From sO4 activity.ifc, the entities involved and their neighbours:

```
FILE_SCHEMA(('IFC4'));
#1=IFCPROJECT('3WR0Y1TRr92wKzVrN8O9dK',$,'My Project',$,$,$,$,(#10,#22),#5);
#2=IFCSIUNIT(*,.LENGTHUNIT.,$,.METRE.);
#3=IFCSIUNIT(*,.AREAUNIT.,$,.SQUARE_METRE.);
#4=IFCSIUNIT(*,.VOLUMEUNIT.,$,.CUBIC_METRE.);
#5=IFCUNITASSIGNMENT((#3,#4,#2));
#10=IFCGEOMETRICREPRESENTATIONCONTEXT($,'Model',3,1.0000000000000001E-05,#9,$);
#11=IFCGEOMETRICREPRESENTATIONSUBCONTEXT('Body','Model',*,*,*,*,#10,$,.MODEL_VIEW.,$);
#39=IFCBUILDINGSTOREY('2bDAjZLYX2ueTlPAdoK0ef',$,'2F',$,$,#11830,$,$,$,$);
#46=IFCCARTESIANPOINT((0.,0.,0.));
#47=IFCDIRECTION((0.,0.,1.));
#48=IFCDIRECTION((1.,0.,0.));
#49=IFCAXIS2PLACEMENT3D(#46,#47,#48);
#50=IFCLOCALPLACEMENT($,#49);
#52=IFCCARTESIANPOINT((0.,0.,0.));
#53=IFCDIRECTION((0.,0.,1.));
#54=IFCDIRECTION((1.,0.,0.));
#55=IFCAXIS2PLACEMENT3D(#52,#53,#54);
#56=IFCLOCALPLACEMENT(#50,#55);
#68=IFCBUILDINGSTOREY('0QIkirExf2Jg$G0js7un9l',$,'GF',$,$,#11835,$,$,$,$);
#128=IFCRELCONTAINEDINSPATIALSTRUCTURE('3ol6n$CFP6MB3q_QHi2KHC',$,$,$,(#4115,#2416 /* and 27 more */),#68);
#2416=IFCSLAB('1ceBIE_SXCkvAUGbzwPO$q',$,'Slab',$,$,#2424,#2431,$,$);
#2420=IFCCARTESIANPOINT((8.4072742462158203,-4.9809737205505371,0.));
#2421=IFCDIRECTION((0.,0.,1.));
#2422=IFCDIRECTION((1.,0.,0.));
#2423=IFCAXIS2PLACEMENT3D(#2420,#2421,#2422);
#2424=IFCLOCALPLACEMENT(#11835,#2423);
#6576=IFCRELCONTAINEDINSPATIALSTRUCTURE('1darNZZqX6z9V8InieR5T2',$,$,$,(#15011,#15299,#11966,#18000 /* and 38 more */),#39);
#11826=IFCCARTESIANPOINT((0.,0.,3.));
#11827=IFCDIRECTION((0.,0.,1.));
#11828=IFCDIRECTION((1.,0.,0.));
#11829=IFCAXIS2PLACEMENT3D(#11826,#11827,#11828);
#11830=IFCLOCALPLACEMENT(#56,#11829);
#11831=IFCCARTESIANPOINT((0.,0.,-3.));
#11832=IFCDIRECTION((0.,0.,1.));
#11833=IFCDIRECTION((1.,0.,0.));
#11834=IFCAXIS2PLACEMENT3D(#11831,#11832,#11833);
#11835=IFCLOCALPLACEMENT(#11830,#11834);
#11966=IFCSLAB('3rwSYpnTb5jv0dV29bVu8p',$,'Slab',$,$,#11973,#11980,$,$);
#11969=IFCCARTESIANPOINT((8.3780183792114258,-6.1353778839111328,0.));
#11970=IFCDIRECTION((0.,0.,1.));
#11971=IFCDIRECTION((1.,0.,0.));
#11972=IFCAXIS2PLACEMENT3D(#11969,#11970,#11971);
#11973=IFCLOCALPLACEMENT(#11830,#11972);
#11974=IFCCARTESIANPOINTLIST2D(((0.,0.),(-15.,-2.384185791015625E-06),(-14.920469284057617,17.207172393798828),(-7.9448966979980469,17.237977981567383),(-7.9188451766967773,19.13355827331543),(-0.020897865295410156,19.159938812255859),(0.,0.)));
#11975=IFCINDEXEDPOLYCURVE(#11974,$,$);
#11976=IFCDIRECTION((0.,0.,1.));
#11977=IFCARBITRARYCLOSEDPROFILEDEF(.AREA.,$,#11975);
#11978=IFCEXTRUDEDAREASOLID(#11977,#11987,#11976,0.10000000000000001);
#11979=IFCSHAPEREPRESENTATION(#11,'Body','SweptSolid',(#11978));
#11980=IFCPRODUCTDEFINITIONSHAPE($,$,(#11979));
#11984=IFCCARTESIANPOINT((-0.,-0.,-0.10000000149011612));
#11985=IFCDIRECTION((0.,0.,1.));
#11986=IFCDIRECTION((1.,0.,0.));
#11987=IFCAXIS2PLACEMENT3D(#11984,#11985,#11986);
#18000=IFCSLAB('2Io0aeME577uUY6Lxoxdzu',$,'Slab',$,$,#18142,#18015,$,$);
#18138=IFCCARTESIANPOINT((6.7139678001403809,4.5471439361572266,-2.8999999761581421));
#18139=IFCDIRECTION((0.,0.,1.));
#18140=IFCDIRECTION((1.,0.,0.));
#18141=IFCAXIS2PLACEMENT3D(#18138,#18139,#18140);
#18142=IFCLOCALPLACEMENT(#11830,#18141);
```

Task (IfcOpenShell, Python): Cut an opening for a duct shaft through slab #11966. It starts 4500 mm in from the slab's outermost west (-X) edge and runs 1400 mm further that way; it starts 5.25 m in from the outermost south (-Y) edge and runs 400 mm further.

```python
import numpy as np
import ifcopenshell
import ifcopenshell.api.feature
import ifcopenshell.api.geometry
import ifcopenshell.api.root
import ifcopenshell.geom
import ifcopenshell.util.placement
import ifcopenshell.util.representation
import ifcopenshell.util.shape
import ifcopenshell.util.unit

model = ifcopenshell.open("sO4 activity.ifc")
unit_scale = ifcopenshell.util.unit.calculate_unit_scale(model)
settings = ifcopenshell.geom.settings()


def volume(element):
    """Net volume in cubic metres, openings subtracted."""
    shape = ifcopenshell.geom.create_shape(settings, element)
    return ifcopenshell.util.shape.get_volume(shape.geometry)


slab = model.by_id(11966)
before = volume(slab)

# Extent in the slab's own axes, in metres. The edges named are its -X and -Y sides.
slab_shape = ifcopenshell.geom.create_shape(settings, slab)
vertices = ifcopenshell.util.shape.get_vertices(slab_shape.geometry)
x_min, y_min, bottom = vertices.min(axis=0)
top = vertices[:, 2].max()

opening = ifcopenshell.api.root.create_entity(model, ifc_class="IfcOpeningElement", name="Duct shaft opening", predefined_type="OPENING")
context = ifcopenshell.util.representation.get_context(model, "Model", "Body", "MODEL_VIEW")
width, depth = 1.4, 0.4
outline = [(0.0, 0.0), (width, 0.0), (width, depth), (0.0, depth), (0.0, 0.0)]
# Overshoot both faces by 50 mm so the cut is clean.
shape = ifcopenshell.api.geometry.add_slab_representation(
    model, context=context, depth=top - bottom + 0.1, polyline=outline
)
ifcopenshell.api.geometry.assign_representation(model, product=opening, representation=shape)

matrix = ifcopenshell.util.placement.get_local_placement(slab.ObjectPlacement)
matrix[:, 3] = matrix @ np.append(np.array([x_min + 4.5, y_min + 5.25, bottom - 0.05]) / unit_scale, 1.0)
ifcopenshell.api.geometry.edit_object_placement(model, product=opening, matrix=matrix, is_si=False)
ifcopenshell.api.feature.add_feature(model, feature=opening, element=slab)

after = volume(slab)

print(f"slab volume {before:.3f} -> {after:.3f} m3")

model.write("sO4 activity-out.ifc")
```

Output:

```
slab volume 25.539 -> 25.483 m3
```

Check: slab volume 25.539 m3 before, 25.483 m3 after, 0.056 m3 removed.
